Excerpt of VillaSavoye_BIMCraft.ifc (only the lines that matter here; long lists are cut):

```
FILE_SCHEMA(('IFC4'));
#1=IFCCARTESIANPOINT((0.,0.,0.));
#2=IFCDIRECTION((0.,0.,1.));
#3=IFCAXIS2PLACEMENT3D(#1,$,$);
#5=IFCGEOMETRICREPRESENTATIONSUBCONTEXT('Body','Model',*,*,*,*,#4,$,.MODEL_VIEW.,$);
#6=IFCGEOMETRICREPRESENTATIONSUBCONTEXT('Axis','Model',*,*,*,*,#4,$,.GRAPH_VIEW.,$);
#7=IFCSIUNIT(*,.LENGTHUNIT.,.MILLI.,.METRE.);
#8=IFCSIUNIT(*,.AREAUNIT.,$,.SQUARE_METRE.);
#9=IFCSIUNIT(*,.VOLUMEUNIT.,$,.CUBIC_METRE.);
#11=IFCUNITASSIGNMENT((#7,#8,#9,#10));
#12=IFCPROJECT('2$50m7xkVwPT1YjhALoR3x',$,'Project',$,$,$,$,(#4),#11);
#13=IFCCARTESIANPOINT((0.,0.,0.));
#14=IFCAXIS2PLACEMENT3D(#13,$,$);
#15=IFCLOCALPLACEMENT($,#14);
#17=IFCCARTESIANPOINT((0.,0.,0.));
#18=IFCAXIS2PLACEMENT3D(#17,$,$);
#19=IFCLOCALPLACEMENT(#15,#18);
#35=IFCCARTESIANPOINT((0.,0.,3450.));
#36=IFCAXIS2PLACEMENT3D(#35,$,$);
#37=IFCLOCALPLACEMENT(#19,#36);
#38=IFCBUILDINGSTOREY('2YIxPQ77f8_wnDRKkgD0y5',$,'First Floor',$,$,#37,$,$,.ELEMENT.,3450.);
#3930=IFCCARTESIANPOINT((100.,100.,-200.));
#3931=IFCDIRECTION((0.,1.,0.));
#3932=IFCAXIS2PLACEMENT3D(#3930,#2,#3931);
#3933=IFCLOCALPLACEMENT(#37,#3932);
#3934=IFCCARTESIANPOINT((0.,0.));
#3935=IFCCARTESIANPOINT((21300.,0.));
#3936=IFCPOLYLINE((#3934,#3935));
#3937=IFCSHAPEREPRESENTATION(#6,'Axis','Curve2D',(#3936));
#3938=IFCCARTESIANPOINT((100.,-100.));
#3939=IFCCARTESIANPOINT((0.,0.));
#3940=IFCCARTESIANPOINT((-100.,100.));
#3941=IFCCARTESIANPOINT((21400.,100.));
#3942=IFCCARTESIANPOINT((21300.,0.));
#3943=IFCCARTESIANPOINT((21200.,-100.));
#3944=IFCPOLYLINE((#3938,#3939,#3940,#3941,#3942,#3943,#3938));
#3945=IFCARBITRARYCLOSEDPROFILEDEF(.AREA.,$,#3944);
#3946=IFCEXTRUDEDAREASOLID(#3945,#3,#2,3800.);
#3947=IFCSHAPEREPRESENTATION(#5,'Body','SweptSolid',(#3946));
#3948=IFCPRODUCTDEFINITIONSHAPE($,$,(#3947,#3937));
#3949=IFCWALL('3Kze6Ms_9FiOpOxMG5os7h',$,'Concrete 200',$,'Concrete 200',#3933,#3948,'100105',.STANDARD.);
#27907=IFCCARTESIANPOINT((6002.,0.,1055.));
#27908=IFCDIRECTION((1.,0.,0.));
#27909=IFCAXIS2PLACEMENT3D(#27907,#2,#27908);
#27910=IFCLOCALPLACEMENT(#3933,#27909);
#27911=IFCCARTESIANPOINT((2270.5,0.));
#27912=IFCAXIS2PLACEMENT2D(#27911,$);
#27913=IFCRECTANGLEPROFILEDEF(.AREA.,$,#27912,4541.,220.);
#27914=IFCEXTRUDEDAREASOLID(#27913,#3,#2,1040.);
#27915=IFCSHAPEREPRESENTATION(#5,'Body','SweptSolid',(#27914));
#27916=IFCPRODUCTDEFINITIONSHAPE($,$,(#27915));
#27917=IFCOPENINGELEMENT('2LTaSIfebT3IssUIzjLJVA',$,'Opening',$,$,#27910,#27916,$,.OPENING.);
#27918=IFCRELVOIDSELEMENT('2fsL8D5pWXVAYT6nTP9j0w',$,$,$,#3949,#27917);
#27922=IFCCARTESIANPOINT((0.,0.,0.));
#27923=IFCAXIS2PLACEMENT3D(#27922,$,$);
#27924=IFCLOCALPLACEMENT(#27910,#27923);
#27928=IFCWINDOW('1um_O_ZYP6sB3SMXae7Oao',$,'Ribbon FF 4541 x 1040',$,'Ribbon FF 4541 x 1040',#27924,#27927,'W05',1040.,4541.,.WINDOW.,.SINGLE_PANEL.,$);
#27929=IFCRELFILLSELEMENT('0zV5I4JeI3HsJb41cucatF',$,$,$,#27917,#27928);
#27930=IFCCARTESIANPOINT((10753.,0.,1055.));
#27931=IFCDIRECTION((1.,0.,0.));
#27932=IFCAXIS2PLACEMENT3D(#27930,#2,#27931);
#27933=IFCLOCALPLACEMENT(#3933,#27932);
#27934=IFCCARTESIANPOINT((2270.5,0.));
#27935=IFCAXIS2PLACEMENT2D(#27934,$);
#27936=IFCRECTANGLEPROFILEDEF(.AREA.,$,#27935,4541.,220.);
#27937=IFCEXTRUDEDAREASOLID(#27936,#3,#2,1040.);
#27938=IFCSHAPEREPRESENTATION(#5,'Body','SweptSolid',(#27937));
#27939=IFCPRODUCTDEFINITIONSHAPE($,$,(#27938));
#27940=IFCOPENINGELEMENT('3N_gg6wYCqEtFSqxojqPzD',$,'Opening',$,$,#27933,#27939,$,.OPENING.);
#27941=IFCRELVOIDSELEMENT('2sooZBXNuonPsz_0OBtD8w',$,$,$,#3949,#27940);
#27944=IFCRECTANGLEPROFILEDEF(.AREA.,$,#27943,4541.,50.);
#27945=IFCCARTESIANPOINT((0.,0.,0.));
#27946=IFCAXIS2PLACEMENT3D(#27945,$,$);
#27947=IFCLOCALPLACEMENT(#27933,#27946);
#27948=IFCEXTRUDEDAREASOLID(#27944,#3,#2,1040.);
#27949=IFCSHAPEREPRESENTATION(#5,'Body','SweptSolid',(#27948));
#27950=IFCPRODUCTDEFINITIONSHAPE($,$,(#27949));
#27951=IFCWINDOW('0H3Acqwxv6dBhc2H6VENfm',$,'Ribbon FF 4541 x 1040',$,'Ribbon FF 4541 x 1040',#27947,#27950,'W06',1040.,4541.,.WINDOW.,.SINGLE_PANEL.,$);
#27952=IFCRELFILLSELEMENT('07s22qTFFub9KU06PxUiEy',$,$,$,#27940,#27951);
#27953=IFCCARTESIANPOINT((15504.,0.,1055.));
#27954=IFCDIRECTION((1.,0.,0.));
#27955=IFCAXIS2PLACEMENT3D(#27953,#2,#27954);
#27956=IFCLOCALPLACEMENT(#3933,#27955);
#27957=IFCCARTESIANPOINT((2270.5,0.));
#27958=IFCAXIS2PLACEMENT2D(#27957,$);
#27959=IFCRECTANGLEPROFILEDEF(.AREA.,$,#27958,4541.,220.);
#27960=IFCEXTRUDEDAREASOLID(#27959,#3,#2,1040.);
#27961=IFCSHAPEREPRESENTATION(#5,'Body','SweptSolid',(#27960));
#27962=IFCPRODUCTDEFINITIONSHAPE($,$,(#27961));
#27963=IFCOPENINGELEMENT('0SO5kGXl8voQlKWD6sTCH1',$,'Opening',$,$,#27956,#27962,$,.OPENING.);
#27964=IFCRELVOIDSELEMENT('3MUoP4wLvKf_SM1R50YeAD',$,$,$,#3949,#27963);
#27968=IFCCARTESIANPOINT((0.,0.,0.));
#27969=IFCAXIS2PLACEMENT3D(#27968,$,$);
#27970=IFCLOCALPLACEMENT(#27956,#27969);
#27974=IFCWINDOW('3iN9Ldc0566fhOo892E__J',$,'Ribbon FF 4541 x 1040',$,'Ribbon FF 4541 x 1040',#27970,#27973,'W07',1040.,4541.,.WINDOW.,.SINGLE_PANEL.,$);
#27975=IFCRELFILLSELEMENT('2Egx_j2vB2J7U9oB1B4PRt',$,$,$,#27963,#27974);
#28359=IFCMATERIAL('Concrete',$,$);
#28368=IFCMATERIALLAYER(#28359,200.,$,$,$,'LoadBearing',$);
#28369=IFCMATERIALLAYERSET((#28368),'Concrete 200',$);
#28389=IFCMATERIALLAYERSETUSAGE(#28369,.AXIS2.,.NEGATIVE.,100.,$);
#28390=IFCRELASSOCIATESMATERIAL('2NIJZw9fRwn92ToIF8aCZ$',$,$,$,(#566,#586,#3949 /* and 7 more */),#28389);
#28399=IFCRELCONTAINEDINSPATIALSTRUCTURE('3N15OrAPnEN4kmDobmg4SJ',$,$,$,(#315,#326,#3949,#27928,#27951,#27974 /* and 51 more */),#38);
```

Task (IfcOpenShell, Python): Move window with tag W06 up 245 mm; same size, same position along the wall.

```python
import numpy as np
import ifcopenshell
import ifcopenshell.api.geometry
import ifcopenshell.util.placement
import ifcopenshell.util.unit

model = ifcopenshell.open("VillaSavoye_BIMCraft.ifc")
unit_scale = ifcopenshell.util.unit.calculate_unit_scale(model)

window = model.by_id(27951)
opening = window.FillsVoids[0].RelatingOpeningElement
dz = 245.0

shift = np.array([0.0, 0.0, dz])
# The window is placed relative to its opening, so it follows when the opening moves.
matrix = ifcopenshell.util.placement.get_local_placement(opening.ObjectPlacement)
matrix[:3, 3] += shift
ifcopenshell.api.geometry.edit_object_placement(
    model, product=opening, matrix=matrix, is_si=False, should_transform_children=True
)

print(f"moved by {dz * unit_scale:+.3f} m")

model.write("VillaSavoye_BIMCraft-out.ifc")
```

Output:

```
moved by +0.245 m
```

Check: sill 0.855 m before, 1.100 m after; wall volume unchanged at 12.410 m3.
